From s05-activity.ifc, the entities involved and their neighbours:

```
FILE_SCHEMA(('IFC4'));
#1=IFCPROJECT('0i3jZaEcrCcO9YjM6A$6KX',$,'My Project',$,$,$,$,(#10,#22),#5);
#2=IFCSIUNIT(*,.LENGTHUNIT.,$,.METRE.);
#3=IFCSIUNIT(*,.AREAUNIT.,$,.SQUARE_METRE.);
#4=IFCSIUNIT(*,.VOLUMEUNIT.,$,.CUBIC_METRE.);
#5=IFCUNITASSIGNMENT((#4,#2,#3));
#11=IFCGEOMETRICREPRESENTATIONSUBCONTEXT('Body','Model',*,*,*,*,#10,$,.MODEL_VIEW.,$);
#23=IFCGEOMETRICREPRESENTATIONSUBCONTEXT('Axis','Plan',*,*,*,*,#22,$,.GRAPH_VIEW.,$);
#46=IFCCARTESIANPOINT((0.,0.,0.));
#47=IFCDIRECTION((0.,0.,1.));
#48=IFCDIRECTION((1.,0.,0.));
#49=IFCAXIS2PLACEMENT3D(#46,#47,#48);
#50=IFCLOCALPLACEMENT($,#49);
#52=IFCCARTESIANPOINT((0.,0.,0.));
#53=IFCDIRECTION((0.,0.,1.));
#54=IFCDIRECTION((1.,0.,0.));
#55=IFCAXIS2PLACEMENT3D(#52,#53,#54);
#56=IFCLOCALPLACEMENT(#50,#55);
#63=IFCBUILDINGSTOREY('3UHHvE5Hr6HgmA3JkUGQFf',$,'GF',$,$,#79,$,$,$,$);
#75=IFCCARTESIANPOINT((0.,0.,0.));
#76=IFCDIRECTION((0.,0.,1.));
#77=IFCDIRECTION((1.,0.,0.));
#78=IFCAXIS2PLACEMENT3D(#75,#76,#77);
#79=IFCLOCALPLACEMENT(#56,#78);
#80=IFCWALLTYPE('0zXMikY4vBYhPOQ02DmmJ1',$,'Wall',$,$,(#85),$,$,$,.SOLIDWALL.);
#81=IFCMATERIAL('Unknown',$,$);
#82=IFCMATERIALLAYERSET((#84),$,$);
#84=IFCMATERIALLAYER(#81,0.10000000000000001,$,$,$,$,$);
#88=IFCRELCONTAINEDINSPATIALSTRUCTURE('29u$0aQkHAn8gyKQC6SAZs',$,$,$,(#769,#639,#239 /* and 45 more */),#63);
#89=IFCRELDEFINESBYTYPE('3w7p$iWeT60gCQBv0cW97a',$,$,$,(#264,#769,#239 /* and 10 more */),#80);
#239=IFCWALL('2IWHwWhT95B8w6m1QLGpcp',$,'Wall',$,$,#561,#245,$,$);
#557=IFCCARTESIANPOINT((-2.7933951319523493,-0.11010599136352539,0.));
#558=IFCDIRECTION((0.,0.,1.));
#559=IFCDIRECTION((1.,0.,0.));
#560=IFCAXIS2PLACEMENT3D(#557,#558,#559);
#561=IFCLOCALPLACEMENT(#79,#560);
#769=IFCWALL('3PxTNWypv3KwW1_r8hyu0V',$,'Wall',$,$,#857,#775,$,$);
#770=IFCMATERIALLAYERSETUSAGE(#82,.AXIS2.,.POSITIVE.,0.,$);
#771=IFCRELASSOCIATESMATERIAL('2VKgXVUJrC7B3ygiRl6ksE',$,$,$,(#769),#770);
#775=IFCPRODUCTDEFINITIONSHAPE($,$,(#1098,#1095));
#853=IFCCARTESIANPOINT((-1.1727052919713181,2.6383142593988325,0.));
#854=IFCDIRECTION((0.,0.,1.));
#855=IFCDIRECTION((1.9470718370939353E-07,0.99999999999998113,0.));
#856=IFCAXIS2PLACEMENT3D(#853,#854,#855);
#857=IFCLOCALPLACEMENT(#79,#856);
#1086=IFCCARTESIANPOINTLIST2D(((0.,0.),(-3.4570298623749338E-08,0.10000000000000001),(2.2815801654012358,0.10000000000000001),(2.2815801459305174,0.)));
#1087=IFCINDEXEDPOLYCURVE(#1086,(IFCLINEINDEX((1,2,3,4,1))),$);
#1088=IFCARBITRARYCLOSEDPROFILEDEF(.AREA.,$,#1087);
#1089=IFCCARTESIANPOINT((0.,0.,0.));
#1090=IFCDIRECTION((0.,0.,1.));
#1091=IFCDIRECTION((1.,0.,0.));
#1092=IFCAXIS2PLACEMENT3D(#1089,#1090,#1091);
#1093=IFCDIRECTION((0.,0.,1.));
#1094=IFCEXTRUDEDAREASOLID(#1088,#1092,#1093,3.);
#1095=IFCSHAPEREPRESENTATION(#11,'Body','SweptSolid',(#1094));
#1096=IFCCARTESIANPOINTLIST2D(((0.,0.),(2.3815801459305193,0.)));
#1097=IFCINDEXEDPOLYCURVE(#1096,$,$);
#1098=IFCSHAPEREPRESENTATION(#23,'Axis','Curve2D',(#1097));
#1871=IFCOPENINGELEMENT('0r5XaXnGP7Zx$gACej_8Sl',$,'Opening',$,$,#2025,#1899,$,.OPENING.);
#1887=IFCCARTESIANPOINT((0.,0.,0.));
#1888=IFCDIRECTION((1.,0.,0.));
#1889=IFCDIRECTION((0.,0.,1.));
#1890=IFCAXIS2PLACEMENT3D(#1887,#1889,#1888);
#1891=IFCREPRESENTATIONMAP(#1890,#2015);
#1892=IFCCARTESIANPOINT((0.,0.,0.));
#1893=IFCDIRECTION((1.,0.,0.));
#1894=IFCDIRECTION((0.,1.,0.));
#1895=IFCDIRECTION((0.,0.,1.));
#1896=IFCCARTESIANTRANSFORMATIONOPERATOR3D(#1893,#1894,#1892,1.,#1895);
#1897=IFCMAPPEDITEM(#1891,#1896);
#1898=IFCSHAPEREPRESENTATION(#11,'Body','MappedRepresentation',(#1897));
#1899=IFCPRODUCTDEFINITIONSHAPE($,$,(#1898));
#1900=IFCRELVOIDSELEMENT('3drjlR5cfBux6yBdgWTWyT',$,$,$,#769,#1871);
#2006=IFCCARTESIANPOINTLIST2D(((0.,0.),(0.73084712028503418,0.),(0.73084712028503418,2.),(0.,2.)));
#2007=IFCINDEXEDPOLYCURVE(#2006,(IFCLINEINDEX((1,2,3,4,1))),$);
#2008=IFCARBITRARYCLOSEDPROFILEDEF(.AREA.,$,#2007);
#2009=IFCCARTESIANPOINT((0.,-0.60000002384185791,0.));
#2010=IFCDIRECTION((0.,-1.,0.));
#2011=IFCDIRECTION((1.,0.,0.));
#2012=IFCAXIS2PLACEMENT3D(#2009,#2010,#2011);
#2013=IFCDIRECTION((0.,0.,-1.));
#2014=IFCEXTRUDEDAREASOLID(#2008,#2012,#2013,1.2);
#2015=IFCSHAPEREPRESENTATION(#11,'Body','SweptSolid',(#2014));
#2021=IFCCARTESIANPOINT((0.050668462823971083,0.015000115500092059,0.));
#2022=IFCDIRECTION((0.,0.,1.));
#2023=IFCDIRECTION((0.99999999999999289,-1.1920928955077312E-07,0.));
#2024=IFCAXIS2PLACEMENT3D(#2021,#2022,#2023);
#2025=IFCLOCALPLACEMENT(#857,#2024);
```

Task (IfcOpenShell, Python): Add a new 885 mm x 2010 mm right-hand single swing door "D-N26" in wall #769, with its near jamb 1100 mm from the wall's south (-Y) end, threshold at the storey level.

```python
import numpy as np
import ifcopenshell
import ifcopenshell.api.feature
import ifcopenshell.api.geometry
import ifcopenshell.api.root
import ifcopenshell.api.spatial
import ifcopenshell.geom
import ifcopenshell.util.element
import ifcopenshell.util.placement
import ifcopenshell.util.representation
import ifcopenshell.util.shape
import ifcopenshell.util.unit

model = ifcopenshell.open("s05-activity.ifc")
unit_scale = ifcopenshell.util.unit.calculate_unit_scale(model)
settings = ifcopenshell.geom.settings()


def volume(element):
    """Net volume in cubic metres, openings subtracted."""
    shape = ifcopenshell.geom.create_shape(settings, element)
    return ifcopenshell.util.shape.get_volume(shape.geometry)


wall = model.by_guid("3PxTNWypv3KwW1_r8hyu0V")
storey = ifcopenshell.util.element.get_container(wall, ifc_class="IfcBuildingStorey")
context = ifcopenshell.util.representation.get_context(model, "Model", "Body", "MODEL_VIEW")
before = volume(wall)

width, height, from_end, sill = 0.885, 2.01, 1.1, 0.0  # metres

# The wall runs along its own X axis, and the end named is its -X end.
wall_shape = ifcopenshell.geom.create_shape(settings, wall)
x, y, z = ifcopenshell.util.shape.get_vertices(wall_shape.geometry).T
start = x.min() + from_end
face, thickness = float(y.min()), float(y.max() - y.min())
wall_matrix = ifcopenshell.util.placement.get_local_placement(wall.ObjectPlacement)
level = ifcopenshell.util.placement.get_local_placement(storey.ObjectPlacement)[2, 3]


def in_wall(x, y):
    """Placement at x, y metres in the wall's axes, at sill height."""
    matrix = wall_matrix.copy()
    matrix[:, 3] = wall_matrix @ np.array([x / unit_scale, y / unit_scale, 0.0, 1.0])
    matrix[2, 3] = level + sill / unit_scale
    return matrix


# Opening: a box that overshoots both wall faces by 50 mm.
opening = ifcopenshell.api.root.create_entity(model, ifc_class="IfcOpeningElement", predefined_type="OPENING")
box = ifcopenshell.api.geometry.add_wall_representation(
    model, context=context, length=width, height=height, thickness=thickness + 0.1
)
ifcopenshell.api.geometry.assign_representation(model, product=opening, representation=box)
ifcopenshell.api.geometry.edit_object_placement(model, product=opening, matrix=in_wall(start, face - 0.05), is_si=False)
ifcopenshell.api.feature.add_feature(model, feature=opening, element=wall)

door = ifcopenshell.api.root.create_entity(model, ifc_class="IfcDoor", name="D-N26", predefined_type="DOOR")
door.OverallWidth, door.OverallHeight = width / unit_scale, height / unit_scale
door.OperationType = "SINGLE_SWING_RIGHT"
body = ifcopenshell.api.geometry.add_door_representation(
    model,
    context=context,
    overall_width=door.OverallWidth,
    overall_height=door.OverallHeight,
    operation_type="SINGLE_SWING_RIGHT",
    lining_properties={"LiningDepth": thickness / unit_scale, "ThresholdDepth": thickness / unit_scale},
)
ifcopenshell.api.geometry.assign_representation(model, product=door, representation=body)
ifcopenshell.api.spatial.assign_container(model, products=[door], relating_structure=storey)
ifcopenshell.api.feature.add_filling(model, opening=opening, element=door)

# The lining spans the wall, so the door starts at the wall face.
ifcopenshell.api.geometry.edit_object_placement(model, product=door, matrix=in_wall(start, face), is_si=False)

after = volume(wall)

print(f"wall volume {before:.3f} -> {after:.3f} m3")

model.write("s05-activity_edited.ifc")
```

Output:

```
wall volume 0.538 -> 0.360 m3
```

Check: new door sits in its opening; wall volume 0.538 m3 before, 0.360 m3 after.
